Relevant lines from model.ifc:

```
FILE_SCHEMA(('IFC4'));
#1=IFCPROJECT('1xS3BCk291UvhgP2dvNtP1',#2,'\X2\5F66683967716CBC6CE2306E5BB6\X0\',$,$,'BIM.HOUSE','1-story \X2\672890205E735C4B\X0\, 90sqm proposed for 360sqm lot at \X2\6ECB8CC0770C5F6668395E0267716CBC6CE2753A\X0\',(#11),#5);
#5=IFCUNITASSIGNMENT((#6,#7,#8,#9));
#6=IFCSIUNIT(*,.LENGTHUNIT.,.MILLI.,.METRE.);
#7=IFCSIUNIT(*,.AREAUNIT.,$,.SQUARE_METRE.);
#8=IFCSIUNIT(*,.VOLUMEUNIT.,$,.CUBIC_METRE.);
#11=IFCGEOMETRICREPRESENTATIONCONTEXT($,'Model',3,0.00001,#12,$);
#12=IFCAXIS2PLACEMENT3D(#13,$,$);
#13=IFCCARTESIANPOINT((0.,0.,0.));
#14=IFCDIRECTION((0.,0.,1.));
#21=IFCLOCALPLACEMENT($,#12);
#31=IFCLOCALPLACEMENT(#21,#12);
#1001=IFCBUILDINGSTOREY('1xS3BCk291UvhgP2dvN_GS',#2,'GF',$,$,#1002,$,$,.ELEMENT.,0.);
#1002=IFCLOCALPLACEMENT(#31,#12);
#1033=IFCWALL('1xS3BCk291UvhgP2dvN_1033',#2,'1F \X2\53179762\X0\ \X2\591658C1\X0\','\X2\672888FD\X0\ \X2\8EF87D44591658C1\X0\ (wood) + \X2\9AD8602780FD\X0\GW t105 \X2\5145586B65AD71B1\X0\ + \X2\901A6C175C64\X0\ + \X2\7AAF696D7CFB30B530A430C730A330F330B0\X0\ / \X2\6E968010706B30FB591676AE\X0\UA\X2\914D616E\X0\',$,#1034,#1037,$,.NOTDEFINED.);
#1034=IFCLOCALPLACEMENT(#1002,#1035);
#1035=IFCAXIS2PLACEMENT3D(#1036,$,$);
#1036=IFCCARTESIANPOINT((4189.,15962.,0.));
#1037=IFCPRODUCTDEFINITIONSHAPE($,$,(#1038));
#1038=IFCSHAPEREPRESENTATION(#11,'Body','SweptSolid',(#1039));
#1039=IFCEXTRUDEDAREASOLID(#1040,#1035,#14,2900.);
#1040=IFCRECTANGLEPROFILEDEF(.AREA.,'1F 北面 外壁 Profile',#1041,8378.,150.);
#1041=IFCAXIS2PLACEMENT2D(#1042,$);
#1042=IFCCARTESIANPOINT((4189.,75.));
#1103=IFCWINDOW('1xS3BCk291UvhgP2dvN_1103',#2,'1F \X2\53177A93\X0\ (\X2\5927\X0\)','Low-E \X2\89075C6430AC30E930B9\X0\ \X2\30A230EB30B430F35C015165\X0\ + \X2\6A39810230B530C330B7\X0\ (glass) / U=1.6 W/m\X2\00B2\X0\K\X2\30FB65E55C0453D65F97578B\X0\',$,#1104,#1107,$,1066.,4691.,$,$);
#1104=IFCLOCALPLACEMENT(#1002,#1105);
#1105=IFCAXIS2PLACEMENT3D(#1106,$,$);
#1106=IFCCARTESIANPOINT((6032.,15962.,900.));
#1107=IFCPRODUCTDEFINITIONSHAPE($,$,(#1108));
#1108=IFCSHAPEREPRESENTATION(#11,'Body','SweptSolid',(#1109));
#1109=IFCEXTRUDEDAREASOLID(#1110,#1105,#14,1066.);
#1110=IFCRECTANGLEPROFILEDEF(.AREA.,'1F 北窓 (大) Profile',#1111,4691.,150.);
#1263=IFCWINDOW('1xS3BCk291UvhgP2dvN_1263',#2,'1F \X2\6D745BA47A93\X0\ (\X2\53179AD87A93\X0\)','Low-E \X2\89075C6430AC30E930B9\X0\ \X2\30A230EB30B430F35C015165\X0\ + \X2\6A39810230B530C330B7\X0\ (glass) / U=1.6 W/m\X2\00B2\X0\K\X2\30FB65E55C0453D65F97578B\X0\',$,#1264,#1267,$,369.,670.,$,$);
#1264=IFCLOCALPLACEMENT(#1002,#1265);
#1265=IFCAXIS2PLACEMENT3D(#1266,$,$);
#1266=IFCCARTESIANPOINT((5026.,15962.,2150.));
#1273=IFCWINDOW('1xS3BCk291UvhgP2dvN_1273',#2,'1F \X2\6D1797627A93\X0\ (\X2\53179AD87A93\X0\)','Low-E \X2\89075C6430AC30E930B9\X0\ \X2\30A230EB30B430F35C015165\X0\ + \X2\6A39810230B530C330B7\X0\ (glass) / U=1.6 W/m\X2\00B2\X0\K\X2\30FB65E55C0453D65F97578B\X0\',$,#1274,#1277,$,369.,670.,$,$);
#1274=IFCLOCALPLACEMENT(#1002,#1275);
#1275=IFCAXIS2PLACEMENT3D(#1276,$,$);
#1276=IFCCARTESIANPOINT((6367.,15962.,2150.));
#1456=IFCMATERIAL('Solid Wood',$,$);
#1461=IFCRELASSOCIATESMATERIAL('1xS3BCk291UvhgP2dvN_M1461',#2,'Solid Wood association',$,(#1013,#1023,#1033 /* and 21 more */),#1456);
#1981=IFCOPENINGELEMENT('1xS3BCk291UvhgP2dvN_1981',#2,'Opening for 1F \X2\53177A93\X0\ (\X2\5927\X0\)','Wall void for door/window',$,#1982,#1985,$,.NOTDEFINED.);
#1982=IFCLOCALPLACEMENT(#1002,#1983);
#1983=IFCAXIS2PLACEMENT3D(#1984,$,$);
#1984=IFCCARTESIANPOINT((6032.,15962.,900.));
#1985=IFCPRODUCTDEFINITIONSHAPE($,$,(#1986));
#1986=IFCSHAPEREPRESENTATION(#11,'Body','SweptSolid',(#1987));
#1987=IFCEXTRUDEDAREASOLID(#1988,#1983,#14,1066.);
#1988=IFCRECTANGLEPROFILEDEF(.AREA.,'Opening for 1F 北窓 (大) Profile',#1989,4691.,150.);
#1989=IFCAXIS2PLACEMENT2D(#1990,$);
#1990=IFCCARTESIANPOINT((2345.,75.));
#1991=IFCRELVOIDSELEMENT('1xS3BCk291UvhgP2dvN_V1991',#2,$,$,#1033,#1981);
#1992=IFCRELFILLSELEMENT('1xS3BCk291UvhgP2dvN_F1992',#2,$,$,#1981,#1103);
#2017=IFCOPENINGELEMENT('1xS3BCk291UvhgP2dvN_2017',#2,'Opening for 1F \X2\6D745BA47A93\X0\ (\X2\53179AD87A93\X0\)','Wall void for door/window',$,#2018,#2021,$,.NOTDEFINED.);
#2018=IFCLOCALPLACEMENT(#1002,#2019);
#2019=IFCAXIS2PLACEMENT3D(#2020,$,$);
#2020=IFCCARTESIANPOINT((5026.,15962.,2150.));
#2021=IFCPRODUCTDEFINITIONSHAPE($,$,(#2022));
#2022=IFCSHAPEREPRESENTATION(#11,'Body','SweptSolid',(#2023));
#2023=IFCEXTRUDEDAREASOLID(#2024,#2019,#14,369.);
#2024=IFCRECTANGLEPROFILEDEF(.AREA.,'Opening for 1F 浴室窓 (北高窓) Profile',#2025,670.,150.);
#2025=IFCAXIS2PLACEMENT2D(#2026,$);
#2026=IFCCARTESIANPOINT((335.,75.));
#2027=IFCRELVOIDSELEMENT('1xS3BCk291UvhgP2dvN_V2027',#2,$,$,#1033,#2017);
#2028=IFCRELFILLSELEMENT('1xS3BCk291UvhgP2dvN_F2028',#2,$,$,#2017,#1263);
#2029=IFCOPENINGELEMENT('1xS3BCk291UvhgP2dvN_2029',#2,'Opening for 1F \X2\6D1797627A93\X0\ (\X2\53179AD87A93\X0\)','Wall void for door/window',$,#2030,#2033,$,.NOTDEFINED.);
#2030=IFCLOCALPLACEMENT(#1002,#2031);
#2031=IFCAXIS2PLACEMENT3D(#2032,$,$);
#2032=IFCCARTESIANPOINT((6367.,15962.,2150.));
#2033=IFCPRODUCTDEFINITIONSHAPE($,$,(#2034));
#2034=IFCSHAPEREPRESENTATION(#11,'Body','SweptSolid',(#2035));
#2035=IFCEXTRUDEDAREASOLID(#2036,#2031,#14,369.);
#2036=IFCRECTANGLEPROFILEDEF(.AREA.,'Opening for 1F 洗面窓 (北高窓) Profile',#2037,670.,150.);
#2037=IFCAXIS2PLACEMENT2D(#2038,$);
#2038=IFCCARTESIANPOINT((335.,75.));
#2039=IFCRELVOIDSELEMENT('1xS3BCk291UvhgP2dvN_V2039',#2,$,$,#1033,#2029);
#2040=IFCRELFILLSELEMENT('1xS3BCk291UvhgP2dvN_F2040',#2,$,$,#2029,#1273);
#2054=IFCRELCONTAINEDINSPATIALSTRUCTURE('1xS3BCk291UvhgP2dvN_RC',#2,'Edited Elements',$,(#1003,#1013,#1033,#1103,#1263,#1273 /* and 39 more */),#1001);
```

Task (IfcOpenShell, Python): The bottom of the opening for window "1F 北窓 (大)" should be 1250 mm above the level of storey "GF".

```python
import numpy as np
import ifcopenshell
import ifcopenshell.api.geometry
import ifcopenshell.geom
import ifcopenshell.util.element
import ifcopenshell.util.placement
import ifcopenshell.util.shape
import ifcopenshell.util.unit

model = ifcopenshell.open("model.ifc")
unit_scale = ifcopenshell.util.unit.calculate_unit_scale(model)

window = model.by_guid("1xS3BCk291UvhgP2dvN_1103")
opening = window.FillsVoids[0].RelatingOpeningElement
storey = ifcopenshell.util.element.get_container(window, ifc_class="IfcBuildingStorey")
level = ifcopenshell.util.placement.get_local_placement(storey.ObjectPlacement)[2, 3]

# The opening's origin need not be at the sill, so measure its lowest point.
shape = ifcopenshell.geom.create_shape(ifcopenshell.geom.settings(), opening)
bottom = ifcopenshell.util.shape.get_shape_bottom_elevation(shape, shape.geometry) / unit_scale
dz = level + 1.25 / unit_scale - bottom

shift = np.array([0.0, 0.0, dz])
# The window is not placed relative to its opening, so move both.
for product in (opening, window):
    matrix = ifcopenshell.util.placement.get_local_placement(product.ObjectPlacement)
    matrix[:3, 3] += shift
    ifcopenshell.api.geometry.edit_object_placement(model, product=product, matrix=matrix, is_si=False)

print(f"moved by {dz * unit_scale:+.3f} m")

model.write("model_rev.ifc")
```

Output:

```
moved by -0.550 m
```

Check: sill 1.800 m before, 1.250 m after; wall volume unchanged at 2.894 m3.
